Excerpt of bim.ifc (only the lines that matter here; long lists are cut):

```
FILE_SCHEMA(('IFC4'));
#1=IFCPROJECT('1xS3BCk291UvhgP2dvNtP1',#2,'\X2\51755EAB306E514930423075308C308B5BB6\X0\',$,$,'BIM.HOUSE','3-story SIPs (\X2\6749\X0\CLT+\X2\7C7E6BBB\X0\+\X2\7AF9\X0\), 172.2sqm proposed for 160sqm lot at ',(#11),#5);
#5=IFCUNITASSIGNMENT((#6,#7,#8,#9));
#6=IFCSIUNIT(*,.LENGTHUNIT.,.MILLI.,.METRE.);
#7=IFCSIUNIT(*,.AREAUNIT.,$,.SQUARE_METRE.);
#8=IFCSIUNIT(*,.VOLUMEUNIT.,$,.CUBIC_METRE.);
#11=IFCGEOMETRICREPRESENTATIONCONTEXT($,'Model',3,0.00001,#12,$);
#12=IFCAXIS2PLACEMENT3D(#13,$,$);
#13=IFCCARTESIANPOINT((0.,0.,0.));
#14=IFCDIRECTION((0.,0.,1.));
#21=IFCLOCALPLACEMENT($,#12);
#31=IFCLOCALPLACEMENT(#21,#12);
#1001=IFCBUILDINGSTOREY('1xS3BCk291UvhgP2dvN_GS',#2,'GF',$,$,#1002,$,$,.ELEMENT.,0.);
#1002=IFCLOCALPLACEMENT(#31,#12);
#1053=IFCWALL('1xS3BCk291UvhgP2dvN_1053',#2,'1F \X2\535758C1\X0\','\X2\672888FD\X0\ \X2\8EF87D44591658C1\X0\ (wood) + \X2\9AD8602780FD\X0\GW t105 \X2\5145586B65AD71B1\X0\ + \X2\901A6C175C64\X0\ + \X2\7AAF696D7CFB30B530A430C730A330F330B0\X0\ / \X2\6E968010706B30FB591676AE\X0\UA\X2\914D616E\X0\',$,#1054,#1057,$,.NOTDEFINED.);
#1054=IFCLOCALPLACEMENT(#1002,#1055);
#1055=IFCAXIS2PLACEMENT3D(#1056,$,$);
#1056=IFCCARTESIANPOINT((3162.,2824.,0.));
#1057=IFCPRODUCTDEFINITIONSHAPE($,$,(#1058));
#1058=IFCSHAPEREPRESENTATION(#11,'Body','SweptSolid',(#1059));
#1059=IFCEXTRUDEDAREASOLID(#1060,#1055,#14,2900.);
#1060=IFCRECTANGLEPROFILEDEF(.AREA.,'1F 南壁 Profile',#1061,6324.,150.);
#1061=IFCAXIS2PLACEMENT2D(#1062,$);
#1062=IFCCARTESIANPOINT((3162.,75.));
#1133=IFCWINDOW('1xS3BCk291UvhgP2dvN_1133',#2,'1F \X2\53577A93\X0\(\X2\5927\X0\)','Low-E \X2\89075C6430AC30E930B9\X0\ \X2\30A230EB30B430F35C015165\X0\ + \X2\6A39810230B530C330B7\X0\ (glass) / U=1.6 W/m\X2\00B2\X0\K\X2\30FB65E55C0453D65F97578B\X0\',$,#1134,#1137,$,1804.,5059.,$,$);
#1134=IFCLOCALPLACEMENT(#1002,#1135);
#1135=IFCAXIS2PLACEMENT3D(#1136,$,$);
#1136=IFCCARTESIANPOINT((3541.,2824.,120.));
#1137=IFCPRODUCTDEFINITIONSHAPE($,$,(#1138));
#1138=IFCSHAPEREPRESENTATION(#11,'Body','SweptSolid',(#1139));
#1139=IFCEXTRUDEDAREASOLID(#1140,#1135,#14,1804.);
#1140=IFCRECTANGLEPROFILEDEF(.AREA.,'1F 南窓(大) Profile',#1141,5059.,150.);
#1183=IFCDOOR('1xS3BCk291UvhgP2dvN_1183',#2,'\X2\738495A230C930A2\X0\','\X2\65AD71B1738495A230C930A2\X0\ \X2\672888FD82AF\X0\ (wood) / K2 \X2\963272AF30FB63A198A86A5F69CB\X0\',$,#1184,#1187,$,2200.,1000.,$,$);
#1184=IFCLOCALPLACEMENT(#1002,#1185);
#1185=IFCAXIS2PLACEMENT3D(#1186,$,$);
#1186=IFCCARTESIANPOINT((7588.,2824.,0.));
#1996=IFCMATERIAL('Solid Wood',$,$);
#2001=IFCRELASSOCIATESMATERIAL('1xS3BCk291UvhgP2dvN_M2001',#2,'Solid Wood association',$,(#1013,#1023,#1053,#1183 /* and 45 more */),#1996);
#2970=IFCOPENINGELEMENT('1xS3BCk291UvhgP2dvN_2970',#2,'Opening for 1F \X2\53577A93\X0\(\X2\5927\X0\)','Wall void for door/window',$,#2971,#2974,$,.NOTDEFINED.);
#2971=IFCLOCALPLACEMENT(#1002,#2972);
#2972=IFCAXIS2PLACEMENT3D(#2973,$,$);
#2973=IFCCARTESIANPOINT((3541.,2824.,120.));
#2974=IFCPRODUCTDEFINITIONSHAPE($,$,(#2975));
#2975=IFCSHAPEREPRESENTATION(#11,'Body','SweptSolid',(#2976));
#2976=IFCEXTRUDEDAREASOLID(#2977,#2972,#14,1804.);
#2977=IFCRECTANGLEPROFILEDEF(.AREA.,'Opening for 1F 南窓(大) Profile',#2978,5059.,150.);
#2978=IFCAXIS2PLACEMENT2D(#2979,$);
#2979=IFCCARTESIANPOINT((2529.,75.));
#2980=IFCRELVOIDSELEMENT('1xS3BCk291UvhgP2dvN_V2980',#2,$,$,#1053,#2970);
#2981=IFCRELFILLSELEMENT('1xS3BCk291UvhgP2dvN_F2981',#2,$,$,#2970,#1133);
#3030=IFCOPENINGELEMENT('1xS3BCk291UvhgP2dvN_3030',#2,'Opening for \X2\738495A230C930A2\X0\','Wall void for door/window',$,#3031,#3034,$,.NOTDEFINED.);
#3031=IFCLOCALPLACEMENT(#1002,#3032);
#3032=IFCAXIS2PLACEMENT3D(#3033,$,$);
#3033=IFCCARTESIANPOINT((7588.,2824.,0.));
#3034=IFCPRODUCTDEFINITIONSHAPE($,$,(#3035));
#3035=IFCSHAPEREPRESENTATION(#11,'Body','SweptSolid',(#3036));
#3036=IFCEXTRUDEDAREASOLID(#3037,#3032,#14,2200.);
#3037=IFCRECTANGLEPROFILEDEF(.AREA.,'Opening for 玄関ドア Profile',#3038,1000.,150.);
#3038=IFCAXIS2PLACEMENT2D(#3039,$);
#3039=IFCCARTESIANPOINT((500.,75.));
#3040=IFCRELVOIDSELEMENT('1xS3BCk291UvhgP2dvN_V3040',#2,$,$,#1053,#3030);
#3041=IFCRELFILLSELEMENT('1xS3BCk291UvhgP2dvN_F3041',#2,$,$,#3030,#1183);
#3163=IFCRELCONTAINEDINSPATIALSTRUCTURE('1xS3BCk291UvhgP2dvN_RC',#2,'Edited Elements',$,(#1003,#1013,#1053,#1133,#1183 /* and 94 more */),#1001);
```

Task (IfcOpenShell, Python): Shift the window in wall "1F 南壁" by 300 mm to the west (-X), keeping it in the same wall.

```python
import ifcopenshell
import ifcopenshell.api.geometry
import ifcopenshell.util.placement

model = ifcopenshell.open("bim.ifc")

window = model.by_guid("1xS3BCk291UvhgP2dvN_1133")
opening = window.FillsVoids[0].RelatingOpeningElement
wall = opening.VoidsElements[0].RelatingBuildingElement

wall_matrix = ifcopenshell.util.placement.get_local_placement(wall.ObjectPlacement)
shift = wall_matrix[:3, 0] * -300.0
before = ifcopenshell.util.placement.get_local_placement(window.ObjectPlacement)[:3, 3].copy()

# The window is not placed relative to its opening, so move both.
for product in (opening, window):
    matrix = ifcopenshell.util.placement.get_local_placement(product.ObjectPlacement)
    matrix[:3, 3] += shift
    ifcopenshell.api.geometry.edit_object_placement(model, product=product, matrix=matrix, is_si=False)

after = ifcopenshell.util.placement.get_local_placement(window.ObjectPlacement)[:3, 3]
print("window moved by", (after - before).round(3) + 0.0)

model.write("bim_rev.ifc")
```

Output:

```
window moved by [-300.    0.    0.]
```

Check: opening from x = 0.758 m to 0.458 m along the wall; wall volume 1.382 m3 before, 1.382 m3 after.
